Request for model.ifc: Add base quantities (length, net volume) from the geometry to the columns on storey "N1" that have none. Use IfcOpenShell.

First a look at what the model holds.

```python
import ifcopenshell
import ifcopenshell.util.element
import ifcopenshell.util.unit

model = ifcopenshell.open("model.ifc")
print(model.schema)
for unit_type in ("LENGTHUNIT", "AREAUNIT", "VOLUMEUNIT"):
    print(unit_type, ifcopenshell.util.unit.calculate_unit_scale(model, unit_type))
storey = next(s for s in model.by_type("IfcBuildingStorey") if s.Name == "N1")
columns = [e for e in ifcopenshell.util.element.get_decomposition(storey) if e.is_a("IfcColumn")]
for e in sorted(columns, key=lambda e: e.id()):
    print(e.id(), e.is_a(), e.Name, list(ifcopenshell.util.element.get_psets(e, qtos_only=True)), sep=" | ")
```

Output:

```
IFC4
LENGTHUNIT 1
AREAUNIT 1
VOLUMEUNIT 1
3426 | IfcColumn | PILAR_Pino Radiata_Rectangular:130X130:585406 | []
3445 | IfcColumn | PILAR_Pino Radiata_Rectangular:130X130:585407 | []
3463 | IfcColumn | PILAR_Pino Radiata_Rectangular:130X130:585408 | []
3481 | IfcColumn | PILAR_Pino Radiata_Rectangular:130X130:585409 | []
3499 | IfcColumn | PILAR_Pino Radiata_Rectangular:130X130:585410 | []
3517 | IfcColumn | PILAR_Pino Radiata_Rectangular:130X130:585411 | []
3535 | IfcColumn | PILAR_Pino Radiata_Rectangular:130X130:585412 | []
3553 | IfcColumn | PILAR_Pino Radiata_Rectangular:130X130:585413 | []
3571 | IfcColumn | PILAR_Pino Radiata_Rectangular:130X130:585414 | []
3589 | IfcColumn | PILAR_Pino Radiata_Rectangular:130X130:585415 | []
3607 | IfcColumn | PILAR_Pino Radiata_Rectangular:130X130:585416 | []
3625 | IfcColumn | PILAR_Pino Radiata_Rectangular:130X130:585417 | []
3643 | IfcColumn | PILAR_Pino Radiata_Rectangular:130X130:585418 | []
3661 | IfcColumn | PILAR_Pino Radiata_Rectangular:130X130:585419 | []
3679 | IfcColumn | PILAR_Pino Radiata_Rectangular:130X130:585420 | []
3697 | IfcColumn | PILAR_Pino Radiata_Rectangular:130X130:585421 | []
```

```python
import ifcopenshell
import ifcopenshell.api.pset
import ifcopenshell.geom
import ifcopenshell.util.element
import ifcopenshell.util.shape
import ifcopenshell.util.unit

model = ifcopenshell.open("model.ifc")
unit_scale = ifcopenshell.util.unit.calculate_unit_scale(model)
volume_scale = ifcopenshell.util.unit.calculate_unit_scale(model, "VOLUMEUNIT")
settings = ifcopenshell.geom.settings()

storey = next(s for s in model.by_type("IfcBuildingStorey") if s.Name == "N1")
columns = [e for e in ifcopenshell.util.element.get_decomposition(storey) if e.is_a("IfcColumn")]

for e in sorted(columns, key=lambda e: e.id()):
    if ifcopenshell.util.element.get_psets(e, qtos_only=True, should_inherit=False):
        continue
    # Geometry comes back in metres, in the element's own axes.
    shape = ifcopenshell.geom.create_shape(settings, e)
    values = {
        "Length": ifcopenshell.util.shape.get_z(shape.geometry) / unit_scale,
        "NetVolume": ifcopenshell.util.shape.get_volume(shape.geometry) / volume_scale,
    }
    qto = ifcopenshell.api.pset.add_qto(model, product=e, name="Qto_ColumnBaseQuantities")
    ifcopenshell.api.pset.edit_qto(model, qto=qto, properties=values)
    print(e.id(), {k: round(v, 3) for k, v in values.items()})

model.write("model_updated.ifc")
```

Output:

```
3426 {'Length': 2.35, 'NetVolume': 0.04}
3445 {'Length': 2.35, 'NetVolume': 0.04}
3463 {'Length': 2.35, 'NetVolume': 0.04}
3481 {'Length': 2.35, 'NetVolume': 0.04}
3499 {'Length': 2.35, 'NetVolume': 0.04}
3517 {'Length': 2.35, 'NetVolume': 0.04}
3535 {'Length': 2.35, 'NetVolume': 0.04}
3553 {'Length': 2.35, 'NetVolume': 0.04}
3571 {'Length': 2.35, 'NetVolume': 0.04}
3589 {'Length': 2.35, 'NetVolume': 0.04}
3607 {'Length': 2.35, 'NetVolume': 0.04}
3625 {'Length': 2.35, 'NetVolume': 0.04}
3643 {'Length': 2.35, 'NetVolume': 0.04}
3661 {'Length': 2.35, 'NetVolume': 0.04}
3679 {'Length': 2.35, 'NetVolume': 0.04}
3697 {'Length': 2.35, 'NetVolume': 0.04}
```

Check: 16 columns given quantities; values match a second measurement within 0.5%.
